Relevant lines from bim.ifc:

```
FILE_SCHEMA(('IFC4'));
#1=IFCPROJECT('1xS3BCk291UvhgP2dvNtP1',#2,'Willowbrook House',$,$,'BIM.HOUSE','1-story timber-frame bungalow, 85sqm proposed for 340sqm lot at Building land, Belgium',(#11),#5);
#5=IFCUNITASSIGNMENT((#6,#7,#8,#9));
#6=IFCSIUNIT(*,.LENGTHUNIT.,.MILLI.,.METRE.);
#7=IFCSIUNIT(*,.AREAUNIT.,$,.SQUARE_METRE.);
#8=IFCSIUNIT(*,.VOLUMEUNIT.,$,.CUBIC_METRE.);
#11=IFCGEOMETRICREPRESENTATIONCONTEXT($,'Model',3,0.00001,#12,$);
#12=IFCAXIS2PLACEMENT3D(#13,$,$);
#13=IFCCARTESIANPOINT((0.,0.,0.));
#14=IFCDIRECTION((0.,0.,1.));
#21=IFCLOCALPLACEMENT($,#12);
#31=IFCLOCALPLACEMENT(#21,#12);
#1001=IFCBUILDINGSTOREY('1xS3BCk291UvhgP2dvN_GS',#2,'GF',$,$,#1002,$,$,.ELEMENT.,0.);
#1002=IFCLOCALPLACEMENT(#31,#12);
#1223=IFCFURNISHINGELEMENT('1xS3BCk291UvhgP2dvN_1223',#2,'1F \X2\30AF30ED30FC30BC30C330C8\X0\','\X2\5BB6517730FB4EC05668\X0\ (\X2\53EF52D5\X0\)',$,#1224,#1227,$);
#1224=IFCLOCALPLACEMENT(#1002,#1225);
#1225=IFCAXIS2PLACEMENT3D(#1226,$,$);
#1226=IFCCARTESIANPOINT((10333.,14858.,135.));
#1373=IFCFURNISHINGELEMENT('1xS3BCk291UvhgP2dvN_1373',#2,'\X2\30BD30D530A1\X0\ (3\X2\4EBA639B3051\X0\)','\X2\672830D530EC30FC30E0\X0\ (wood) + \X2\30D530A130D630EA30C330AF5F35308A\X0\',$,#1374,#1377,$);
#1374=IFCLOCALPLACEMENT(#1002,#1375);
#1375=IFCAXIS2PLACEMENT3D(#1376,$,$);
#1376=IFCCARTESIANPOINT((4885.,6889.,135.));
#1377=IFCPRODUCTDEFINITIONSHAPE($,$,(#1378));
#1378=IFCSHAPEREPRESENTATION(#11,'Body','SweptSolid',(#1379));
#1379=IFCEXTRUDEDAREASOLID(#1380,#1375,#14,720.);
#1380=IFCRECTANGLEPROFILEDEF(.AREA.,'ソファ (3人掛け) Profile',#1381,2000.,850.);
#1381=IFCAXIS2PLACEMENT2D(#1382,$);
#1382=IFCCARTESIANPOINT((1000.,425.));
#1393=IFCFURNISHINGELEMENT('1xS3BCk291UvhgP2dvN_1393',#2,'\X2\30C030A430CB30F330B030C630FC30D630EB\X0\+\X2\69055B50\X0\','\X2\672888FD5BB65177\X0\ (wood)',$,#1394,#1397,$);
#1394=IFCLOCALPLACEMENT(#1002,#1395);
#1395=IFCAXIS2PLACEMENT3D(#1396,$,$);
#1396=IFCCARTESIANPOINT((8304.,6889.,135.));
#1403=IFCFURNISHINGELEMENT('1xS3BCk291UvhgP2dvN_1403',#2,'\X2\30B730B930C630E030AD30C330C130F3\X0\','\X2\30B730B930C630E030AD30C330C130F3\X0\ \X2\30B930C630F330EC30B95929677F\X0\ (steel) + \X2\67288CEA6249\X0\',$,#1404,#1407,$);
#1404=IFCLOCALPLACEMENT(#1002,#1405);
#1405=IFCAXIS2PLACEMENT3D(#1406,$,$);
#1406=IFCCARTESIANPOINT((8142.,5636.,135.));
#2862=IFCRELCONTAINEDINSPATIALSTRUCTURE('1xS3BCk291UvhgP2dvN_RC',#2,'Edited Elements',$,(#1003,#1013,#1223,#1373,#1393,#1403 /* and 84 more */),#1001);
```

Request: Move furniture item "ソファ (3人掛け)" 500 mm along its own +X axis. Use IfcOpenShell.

```python
import ifcopenshell
import ifcopenshell.api.geometry
import ifcopenshell.util.placement

model = ifcopenshell.open("bim.ifc")

item = model.by_guid("1xS3BCk291UvhgP2dvN_1373")
matrix = ifcopenshell.util.placement.get_local_placement(item.ObjectPlacement)
matrix[:3, 3] += matrix[:3, 0] * 500.0
ifcopenshell.api.geometry.edit_object_placement(model, product=item, matrix=matrix, is_si=False)

print(ifcopenshell.util.placement.get_local_placement(item.ObjectPlacement).round(3) + 0.0)

model.write("bim-out.ifc")
```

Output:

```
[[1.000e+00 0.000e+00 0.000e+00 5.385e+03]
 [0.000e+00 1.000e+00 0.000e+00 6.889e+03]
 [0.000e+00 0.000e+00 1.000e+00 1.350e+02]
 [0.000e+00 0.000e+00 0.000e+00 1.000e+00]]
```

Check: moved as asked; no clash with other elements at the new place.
